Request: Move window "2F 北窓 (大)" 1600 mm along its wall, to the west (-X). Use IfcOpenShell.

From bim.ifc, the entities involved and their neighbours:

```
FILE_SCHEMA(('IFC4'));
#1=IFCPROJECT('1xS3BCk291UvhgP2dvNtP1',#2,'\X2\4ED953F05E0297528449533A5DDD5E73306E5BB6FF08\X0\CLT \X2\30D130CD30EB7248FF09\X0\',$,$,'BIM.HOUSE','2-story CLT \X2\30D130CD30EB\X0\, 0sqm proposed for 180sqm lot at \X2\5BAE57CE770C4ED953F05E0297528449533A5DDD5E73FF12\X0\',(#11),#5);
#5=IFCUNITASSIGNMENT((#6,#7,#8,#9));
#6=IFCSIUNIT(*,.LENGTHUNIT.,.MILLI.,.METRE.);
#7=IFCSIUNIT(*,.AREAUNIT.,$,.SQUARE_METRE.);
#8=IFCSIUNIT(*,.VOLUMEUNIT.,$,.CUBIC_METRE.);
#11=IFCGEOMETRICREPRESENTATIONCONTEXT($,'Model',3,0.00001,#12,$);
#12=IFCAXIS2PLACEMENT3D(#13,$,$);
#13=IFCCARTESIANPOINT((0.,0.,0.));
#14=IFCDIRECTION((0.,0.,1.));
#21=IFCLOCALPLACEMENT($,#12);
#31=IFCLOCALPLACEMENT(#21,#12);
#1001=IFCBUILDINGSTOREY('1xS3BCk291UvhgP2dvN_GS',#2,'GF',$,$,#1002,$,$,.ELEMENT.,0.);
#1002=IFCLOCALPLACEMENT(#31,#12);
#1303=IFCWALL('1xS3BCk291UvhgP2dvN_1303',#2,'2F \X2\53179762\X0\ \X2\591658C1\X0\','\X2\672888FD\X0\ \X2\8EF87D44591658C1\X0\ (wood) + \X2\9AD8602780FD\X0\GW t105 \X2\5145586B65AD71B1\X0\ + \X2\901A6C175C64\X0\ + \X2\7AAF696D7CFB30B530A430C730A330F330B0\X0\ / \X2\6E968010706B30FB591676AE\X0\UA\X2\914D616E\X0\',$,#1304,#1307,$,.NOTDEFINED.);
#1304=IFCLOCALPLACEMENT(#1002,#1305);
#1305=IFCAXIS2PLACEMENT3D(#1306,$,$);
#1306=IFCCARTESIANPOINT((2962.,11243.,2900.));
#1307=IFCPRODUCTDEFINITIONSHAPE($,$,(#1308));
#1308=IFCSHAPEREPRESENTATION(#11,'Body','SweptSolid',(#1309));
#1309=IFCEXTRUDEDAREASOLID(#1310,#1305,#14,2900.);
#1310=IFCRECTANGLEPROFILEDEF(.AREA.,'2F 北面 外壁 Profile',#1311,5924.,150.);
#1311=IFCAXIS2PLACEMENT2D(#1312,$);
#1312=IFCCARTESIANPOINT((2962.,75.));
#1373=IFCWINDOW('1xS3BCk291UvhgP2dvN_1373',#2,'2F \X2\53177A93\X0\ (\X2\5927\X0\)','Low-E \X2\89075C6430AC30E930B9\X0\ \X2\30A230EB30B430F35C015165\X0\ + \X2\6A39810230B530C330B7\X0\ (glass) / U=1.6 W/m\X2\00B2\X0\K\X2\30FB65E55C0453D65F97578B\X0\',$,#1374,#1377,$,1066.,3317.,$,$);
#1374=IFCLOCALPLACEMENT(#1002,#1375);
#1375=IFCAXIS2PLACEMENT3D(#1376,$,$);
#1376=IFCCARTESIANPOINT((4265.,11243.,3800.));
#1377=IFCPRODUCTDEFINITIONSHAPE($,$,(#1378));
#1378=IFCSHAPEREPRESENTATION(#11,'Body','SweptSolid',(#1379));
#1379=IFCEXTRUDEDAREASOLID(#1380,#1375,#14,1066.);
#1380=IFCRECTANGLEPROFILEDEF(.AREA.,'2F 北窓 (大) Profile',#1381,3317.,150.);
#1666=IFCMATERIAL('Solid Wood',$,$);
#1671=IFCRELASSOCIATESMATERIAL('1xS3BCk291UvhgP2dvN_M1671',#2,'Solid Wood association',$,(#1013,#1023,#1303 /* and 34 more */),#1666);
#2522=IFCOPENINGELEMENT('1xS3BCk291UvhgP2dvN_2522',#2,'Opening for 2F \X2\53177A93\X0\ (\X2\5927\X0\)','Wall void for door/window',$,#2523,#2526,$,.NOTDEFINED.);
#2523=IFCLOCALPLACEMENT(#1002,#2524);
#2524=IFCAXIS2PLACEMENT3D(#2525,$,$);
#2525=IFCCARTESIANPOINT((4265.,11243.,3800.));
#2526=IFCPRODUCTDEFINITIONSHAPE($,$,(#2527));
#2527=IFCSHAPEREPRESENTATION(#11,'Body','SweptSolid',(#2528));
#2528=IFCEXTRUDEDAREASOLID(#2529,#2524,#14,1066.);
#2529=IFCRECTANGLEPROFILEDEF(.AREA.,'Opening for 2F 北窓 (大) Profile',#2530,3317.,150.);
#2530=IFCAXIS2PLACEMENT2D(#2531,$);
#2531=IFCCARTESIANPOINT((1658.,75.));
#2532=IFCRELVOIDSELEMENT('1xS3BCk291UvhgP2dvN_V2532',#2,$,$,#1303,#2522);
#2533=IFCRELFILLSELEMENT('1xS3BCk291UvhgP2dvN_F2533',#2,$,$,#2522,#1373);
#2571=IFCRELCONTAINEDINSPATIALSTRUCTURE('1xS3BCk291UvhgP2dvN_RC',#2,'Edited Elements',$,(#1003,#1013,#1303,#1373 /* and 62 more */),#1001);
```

```python
import ifcopenshell
import ifcopenshell.api.geometry
import ifcopenshell.util.placement
import ifcopenshell.util.unit

model = ifcopenshell.open("bim.ifc")
unit_scale = ifcopenshell.util.unit.calculate_unit_scale(model)

window = model.by_id(1373)
opening = window.FillsVoids[0].RelatingOpeningElement
wall = opening.VoidsElements[0].RelatingBuildingElement

wall_matrix = ifcopenshell.util.placement.get_local_placement(wall.ObjectPlacement)
shift = wall_matrix[:3, 0] * -1.6 / unit_scale
before = ifcopenshell.util.placement.get_local_placement(window.ObjectPlacement)[:3, 3].copy()

# The window is not placed relative to its opening, so move both.
for product in (opening, window):
    matrix = ifcopenshell.util.placement.get_local_placement(product.ObjectPlacement)
    matrix[:3, 3] += shift
    ifcopenshell.api.geometry.edit_object_placement(model, product=product, matrix=matrix, is_si=False)

after = ifcopenshell.util.placement.get_local_placement(window.ObjectPlacement)[:3, 3]
print("window moved by", (after - before).round(3) + 0.0)

model.write("bim_rev.ifc")
```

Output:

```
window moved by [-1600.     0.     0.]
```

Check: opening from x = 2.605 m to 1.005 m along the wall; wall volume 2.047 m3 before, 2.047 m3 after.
